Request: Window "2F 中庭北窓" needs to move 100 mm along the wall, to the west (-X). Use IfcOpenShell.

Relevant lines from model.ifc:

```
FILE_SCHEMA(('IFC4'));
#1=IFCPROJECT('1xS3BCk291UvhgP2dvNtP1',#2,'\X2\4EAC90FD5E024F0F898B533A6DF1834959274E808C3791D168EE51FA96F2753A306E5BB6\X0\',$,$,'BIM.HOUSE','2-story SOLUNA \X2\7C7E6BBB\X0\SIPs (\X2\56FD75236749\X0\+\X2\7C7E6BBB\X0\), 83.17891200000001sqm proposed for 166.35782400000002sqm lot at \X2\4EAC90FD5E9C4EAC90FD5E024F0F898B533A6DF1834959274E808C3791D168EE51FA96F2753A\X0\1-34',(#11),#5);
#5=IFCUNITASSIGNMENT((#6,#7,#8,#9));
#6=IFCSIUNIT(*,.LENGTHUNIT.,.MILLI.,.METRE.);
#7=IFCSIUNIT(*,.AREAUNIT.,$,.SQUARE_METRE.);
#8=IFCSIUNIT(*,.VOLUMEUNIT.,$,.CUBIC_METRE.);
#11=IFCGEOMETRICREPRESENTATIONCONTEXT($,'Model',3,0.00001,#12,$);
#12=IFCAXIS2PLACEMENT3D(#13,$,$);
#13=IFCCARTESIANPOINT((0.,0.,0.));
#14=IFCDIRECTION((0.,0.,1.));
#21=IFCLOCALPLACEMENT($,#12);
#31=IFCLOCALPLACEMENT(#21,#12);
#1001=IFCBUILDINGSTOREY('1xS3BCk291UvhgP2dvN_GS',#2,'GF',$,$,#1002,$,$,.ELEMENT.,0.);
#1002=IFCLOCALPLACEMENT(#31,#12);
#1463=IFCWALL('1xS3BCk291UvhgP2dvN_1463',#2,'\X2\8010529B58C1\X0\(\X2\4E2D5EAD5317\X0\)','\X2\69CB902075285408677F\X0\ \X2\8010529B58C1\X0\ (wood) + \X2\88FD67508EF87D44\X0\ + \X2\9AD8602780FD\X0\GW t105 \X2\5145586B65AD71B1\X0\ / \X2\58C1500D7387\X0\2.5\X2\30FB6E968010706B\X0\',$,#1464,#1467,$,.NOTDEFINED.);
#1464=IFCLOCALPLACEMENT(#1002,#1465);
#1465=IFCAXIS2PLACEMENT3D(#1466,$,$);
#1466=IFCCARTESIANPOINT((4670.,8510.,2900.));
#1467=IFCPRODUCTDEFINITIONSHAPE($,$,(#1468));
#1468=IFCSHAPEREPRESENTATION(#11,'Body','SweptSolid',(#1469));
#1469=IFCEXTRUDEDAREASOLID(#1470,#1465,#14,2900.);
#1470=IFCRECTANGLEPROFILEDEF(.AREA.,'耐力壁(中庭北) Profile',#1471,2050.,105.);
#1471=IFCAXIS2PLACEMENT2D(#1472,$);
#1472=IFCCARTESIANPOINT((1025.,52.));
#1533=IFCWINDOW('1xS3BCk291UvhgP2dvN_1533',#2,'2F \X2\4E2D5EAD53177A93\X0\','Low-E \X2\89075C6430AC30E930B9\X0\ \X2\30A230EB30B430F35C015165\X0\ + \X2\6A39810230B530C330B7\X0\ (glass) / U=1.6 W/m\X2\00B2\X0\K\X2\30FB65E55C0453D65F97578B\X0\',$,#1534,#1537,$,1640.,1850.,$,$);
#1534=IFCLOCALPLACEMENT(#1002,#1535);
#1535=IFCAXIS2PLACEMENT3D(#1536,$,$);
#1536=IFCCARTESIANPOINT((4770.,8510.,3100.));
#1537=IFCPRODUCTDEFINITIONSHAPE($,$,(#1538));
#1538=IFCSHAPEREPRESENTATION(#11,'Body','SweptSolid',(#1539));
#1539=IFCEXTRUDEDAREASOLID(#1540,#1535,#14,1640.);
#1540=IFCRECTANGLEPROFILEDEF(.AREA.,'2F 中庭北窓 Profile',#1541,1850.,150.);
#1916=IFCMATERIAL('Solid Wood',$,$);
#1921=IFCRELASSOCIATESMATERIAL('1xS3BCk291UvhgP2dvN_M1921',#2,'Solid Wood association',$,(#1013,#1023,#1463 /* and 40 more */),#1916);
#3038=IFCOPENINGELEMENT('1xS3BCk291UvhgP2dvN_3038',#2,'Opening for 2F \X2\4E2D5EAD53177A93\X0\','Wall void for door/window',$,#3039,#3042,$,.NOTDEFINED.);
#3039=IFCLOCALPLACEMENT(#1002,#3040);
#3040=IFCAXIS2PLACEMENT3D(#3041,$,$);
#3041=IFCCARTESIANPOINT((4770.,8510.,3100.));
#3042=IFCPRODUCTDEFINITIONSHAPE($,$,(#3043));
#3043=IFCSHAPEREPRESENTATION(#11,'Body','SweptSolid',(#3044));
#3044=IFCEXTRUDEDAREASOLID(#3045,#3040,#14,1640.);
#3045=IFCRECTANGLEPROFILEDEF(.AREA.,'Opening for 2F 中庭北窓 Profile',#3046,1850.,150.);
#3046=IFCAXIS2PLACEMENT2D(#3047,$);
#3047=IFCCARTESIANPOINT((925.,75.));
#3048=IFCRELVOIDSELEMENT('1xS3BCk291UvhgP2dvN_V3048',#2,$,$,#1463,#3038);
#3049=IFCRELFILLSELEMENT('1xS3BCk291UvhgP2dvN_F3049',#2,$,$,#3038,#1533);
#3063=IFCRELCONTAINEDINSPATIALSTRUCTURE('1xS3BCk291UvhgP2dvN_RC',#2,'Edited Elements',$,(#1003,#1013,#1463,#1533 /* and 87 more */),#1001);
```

```python
import ifcopenshell
import ifcopenshell.api.geometry
import ifcopenshell.util.placement

model = ifcopenshell.open("model.ifc")

window = model.by_guid("1xS3BCk291UvhgP2dvN_1533")
opening = window.FillsVoids[0].RelatingOpeningElement
wall = opening.VoidsElements[0].RelatingBuildingElement

wall_matrix = ifcopenshell.util.placement.get_local_placement(wall.ObjectPlacement)
shift = wall_matrix[:3, 0] * -100.0
before = ifcopenshell.util.placement.get_local_placement(window.ObjectPlacement)[:3, 3].copy()

# The window is not placed relative to its opening, so move both.
for product in (opening, window):
    matrix = ifcopenshell.util.placement.get_local_placement(product.ObjectPlacement)
    matrix[:3, 3] += shift
    ifcopenshell.api.geometry.edit_object_placement(model, product=product, matrix=matrix, is_si=False)

after = ifcopenshell.util.placement.get_local_placement(window.ObjectPlacement)[:3, 3]
print("window moved by", (after - before).round(3) + 0.0)

model.write("model-out.ifc")
```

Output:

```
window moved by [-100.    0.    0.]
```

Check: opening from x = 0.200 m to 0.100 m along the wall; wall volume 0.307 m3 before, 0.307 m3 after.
